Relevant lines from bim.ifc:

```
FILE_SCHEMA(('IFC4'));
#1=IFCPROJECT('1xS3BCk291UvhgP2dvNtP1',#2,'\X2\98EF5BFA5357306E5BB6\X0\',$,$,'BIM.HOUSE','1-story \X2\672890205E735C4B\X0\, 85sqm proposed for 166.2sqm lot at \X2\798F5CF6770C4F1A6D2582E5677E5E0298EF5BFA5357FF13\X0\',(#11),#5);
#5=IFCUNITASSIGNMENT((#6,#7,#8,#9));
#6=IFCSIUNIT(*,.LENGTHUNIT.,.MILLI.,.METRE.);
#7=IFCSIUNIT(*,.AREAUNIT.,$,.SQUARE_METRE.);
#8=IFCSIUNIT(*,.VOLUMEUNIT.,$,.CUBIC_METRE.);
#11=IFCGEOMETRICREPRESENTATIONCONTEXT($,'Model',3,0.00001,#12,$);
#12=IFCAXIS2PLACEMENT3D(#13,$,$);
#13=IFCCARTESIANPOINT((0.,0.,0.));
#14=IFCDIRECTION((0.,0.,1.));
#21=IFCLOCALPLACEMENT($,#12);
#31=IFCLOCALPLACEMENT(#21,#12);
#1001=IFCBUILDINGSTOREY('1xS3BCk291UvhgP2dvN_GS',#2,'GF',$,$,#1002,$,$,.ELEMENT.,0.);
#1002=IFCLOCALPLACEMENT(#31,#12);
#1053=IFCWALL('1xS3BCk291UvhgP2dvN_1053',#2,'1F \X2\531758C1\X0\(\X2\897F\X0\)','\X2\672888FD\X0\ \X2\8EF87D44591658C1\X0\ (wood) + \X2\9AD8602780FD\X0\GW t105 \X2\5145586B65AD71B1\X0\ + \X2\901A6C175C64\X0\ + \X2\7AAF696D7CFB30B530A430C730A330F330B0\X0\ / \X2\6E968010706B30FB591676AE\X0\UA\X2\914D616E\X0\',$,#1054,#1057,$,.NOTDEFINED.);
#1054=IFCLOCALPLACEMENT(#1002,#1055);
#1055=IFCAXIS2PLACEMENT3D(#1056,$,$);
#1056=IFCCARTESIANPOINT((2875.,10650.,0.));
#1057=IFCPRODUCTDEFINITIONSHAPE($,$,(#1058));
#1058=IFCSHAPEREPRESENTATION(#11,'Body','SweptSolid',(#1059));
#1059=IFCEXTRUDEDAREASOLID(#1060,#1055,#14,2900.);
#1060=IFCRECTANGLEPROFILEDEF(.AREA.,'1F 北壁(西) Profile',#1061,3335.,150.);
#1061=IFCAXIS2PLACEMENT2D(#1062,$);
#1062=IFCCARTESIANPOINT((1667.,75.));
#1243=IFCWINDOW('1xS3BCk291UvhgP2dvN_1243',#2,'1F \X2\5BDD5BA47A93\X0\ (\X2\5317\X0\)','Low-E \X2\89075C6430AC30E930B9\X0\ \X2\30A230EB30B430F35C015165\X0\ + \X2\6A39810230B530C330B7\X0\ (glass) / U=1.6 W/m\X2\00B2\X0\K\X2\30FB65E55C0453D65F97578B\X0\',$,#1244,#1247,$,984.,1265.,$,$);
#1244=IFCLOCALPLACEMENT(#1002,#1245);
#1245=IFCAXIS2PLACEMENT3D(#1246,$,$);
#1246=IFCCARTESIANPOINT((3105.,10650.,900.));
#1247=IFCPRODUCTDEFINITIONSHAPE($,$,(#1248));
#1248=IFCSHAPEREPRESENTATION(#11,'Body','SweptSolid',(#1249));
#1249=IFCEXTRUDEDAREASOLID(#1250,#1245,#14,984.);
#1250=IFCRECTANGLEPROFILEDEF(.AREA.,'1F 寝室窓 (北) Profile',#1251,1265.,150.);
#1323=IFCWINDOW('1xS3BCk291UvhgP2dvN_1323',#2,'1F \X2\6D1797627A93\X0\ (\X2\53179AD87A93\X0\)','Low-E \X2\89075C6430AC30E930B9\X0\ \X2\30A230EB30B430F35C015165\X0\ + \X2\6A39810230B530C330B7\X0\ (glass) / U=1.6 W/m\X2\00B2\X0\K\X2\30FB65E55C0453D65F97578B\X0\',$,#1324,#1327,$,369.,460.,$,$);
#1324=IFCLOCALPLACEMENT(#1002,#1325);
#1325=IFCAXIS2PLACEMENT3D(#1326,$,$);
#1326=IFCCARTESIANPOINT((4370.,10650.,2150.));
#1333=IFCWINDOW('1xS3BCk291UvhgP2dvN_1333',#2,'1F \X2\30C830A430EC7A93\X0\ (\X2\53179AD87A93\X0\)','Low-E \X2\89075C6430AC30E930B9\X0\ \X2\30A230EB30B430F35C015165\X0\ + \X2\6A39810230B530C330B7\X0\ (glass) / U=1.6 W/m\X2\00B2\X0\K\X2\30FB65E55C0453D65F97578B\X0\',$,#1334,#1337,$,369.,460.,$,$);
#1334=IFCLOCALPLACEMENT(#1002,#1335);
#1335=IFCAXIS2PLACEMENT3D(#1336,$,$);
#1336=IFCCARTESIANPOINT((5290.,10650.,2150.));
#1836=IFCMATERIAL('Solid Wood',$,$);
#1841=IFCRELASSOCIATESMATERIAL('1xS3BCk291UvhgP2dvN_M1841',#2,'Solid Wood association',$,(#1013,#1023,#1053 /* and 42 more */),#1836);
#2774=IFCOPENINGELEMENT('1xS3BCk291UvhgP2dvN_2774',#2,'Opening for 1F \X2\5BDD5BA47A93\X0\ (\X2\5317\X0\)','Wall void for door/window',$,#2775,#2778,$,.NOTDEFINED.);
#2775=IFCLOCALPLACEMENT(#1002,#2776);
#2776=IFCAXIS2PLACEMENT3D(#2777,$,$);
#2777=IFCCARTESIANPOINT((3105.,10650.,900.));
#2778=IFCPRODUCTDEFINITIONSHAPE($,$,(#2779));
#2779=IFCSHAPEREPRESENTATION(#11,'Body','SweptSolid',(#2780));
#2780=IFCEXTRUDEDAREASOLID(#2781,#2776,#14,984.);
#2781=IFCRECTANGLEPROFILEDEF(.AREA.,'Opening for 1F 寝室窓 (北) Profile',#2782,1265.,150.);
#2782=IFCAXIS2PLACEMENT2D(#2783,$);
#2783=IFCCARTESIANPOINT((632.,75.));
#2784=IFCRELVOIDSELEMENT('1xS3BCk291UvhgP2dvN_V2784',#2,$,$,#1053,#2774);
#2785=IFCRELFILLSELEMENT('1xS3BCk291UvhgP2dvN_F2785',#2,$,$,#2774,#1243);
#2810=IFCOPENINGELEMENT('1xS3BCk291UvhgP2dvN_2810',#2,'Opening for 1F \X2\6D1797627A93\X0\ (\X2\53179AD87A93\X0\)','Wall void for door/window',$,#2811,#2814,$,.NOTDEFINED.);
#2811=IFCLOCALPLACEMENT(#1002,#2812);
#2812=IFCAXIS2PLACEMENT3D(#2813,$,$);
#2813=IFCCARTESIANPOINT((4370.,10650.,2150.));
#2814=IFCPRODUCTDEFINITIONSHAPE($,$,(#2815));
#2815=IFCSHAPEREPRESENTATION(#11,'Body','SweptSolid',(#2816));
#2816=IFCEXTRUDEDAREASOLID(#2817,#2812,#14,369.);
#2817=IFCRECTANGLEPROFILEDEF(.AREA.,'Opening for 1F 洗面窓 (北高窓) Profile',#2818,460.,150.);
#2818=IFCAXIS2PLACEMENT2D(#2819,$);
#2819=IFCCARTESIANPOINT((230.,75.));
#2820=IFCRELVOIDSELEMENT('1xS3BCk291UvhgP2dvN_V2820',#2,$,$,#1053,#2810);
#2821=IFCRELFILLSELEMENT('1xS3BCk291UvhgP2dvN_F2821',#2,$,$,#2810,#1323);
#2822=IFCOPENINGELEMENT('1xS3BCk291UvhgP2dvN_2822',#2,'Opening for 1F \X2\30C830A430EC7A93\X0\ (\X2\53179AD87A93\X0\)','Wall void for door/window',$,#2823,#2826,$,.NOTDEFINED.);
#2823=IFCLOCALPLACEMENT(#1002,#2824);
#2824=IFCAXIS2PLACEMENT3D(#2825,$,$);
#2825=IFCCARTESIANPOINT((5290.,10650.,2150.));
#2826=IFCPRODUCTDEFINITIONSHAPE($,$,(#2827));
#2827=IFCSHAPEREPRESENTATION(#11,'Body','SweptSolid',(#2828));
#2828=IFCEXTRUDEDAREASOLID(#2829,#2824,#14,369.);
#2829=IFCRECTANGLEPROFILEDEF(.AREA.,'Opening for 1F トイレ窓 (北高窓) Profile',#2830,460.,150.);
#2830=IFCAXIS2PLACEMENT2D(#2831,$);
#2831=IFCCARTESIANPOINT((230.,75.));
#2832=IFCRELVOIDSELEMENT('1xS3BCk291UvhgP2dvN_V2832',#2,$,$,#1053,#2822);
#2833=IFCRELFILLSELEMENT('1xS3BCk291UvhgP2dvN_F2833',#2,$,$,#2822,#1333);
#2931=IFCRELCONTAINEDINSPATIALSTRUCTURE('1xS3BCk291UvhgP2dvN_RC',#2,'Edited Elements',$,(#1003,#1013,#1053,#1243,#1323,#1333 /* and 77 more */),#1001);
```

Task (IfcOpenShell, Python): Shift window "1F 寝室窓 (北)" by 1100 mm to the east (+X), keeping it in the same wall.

```python
import ifcopenshell
import ifcopenshell.api.geometry
import ifcopenshell.util.placement

model = ifcopenshell.open("bim.ifc")

window = model.by_guid("1xS3BCk291UvhgP2dvN_1243")
opening = window.FillsVoids[0].RelatingOpeningElement
wall = opening.VoidsElements[0].RelatingBuildingElement

wall_matrix = ifcopenshell.util.placement.get_local_placement(wall.ObjectPlacement)
shift = wall_matrix[:3, 0] * 1100.0
before = ifcopenshell.util.placement.get_local_placement(window.ObjectPlacement)[:3, 3].copy()

# The window is not placed relative to its opening, so move both.
for product in (opening, window):
    matrix = ifcopenshell.util.placement.get_local_placement(product.ObjectPlacement)
    matrix[:3, 3] += shift
    ifcopenshell.api.geometry.edit_object_placement(model, product=product, matrix=matrix, is_si=False)

after = ifcopenshell.util.placement.get_local_placement(window.ObjectPlacement)[:3, 3]
print("window moved by", (after - before).round(3) + 0.0)

model.write("bim_edited.ifc")
```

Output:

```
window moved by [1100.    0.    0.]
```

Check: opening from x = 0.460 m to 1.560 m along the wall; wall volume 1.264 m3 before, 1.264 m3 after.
